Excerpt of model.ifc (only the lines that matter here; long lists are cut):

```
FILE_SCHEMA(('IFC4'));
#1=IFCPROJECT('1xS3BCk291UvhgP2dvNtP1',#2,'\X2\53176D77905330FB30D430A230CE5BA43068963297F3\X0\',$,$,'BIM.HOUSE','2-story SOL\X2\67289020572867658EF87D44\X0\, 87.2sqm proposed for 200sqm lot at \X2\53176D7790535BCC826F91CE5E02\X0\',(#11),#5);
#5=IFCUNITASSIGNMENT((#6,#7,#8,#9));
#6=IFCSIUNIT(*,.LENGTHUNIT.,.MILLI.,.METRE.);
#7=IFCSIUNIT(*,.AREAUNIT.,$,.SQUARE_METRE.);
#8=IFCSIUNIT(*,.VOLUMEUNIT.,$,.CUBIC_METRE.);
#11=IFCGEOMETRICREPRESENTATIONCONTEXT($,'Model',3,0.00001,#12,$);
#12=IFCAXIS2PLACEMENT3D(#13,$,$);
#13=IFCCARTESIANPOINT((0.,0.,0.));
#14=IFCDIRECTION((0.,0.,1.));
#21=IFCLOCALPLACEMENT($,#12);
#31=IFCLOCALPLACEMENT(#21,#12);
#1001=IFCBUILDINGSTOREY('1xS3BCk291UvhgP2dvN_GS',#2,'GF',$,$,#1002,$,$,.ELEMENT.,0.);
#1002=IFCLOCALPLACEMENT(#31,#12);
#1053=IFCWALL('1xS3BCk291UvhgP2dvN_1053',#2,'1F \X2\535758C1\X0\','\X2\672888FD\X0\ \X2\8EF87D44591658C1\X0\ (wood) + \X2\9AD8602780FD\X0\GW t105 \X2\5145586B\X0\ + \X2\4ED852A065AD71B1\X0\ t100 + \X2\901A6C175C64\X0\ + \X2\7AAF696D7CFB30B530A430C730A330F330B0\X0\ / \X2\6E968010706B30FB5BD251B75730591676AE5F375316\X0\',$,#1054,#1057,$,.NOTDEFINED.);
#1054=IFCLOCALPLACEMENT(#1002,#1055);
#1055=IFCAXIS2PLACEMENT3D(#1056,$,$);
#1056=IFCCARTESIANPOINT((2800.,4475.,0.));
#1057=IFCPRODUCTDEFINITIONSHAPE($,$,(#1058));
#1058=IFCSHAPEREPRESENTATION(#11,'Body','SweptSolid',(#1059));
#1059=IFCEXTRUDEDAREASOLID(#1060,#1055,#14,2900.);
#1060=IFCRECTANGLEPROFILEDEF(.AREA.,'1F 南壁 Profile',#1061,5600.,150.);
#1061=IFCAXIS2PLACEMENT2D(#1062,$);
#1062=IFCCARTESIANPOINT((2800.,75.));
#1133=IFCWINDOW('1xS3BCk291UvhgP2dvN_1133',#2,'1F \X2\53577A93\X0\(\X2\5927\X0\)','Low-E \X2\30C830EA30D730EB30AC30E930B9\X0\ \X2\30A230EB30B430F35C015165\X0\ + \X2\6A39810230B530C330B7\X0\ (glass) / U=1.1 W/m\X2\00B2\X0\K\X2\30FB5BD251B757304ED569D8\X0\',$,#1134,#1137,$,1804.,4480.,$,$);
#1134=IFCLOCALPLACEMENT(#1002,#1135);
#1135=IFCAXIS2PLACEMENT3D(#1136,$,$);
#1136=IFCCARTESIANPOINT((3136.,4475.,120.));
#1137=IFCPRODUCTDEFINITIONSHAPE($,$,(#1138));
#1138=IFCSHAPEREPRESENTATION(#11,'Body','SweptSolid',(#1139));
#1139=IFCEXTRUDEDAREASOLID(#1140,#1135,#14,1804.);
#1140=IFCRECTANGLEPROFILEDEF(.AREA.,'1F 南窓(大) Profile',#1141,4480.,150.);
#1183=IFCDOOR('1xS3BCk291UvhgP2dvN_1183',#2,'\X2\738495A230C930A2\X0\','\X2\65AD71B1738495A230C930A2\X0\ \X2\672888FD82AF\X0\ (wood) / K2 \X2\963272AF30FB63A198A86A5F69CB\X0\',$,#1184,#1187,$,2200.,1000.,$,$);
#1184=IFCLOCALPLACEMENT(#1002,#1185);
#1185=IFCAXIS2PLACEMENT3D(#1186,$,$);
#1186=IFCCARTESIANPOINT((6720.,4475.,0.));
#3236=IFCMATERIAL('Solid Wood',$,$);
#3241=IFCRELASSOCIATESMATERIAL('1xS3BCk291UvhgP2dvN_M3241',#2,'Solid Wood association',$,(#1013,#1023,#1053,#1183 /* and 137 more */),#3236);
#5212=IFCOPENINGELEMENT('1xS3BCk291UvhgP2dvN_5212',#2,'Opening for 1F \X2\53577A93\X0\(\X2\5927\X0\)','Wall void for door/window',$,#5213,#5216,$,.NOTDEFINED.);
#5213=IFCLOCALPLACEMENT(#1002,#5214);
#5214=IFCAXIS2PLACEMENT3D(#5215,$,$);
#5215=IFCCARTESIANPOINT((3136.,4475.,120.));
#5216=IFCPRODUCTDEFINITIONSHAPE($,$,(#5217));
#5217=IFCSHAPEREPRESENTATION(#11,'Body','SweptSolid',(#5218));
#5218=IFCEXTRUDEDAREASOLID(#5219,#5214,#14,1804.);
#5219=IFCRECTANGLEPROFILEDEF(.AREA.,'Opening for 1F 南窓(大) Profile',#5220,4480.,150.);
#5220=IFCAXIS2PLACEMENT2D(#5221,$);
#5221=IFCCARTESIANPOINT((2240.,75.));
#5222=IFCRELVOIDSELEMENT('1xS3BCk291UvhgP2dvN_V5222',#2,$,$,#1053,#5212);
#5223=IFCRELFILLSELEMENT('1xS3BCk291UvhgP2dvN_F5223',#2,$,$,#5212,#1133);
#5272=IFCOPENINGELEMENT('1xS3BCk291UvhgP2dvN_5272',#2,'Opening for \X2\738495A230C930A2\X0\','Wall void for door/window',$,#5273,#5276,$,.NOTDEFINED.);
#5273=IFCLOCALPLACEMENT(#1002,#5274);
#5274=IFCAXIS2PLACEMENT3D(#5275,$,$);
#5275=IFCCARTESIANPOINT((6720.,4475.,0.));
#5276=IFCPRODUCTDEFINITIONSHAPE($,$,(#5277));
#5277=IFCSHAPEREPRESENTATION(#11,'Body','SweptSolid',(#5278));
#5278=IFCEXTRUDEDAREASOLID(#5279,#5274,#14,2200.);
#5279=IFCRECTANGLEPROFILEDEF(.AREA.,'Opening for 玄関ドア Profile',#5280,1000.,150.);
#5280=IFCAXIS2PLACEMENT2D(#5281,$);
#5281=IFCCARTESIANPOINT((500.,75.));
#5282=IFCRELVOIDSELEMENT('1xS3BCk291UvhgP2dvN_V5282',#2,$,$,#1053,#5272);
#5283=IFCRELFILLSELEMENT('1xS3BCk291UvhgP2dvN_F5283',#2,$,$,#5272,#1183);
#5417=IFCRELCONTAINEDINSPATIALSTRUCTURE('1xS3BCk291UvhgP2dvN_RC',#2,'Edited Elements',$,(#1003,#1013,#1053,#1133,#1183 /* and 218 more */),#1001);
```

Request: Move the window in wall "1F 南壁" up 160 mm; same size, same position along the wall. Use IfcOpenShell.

```python
import numpy as np
import ifcopenshell
import ifcopenshell.api.geometry
import ifcopenshell.util.placement
import ifcopenshell.util.unit

model = ifcopenshell.open("model.ifc")
unit_scale = ifcopenshell.util.unit.calculate_unit_scale(model)

window = model.by_guid("1xS3BCk291UvhgP2dvN_1133")
opening = window.FillsVoids[0].RelatingOpeningElement
dz = 0.16 / unit_scale

shift = np.array([0.0, 0.0, dz])
# The window is not placed relative to its opening, so move both.
for product in (opening, window):
    matrix = ifcopenshell.util.placement.get_local_placement(product.ObjectPlacement)
    matrix[:3, 3] += shift
    ifcopenshell.api.geometry.edit_object_placement(model, product=product, matrix=matrix, is_si=False)

print(f"moved by {dz * unit_scale:+.3f} m")

model.write("model_updated.ifc")
```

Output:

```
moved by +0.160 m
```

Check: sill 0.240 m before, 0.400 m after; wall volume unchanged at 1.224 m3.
